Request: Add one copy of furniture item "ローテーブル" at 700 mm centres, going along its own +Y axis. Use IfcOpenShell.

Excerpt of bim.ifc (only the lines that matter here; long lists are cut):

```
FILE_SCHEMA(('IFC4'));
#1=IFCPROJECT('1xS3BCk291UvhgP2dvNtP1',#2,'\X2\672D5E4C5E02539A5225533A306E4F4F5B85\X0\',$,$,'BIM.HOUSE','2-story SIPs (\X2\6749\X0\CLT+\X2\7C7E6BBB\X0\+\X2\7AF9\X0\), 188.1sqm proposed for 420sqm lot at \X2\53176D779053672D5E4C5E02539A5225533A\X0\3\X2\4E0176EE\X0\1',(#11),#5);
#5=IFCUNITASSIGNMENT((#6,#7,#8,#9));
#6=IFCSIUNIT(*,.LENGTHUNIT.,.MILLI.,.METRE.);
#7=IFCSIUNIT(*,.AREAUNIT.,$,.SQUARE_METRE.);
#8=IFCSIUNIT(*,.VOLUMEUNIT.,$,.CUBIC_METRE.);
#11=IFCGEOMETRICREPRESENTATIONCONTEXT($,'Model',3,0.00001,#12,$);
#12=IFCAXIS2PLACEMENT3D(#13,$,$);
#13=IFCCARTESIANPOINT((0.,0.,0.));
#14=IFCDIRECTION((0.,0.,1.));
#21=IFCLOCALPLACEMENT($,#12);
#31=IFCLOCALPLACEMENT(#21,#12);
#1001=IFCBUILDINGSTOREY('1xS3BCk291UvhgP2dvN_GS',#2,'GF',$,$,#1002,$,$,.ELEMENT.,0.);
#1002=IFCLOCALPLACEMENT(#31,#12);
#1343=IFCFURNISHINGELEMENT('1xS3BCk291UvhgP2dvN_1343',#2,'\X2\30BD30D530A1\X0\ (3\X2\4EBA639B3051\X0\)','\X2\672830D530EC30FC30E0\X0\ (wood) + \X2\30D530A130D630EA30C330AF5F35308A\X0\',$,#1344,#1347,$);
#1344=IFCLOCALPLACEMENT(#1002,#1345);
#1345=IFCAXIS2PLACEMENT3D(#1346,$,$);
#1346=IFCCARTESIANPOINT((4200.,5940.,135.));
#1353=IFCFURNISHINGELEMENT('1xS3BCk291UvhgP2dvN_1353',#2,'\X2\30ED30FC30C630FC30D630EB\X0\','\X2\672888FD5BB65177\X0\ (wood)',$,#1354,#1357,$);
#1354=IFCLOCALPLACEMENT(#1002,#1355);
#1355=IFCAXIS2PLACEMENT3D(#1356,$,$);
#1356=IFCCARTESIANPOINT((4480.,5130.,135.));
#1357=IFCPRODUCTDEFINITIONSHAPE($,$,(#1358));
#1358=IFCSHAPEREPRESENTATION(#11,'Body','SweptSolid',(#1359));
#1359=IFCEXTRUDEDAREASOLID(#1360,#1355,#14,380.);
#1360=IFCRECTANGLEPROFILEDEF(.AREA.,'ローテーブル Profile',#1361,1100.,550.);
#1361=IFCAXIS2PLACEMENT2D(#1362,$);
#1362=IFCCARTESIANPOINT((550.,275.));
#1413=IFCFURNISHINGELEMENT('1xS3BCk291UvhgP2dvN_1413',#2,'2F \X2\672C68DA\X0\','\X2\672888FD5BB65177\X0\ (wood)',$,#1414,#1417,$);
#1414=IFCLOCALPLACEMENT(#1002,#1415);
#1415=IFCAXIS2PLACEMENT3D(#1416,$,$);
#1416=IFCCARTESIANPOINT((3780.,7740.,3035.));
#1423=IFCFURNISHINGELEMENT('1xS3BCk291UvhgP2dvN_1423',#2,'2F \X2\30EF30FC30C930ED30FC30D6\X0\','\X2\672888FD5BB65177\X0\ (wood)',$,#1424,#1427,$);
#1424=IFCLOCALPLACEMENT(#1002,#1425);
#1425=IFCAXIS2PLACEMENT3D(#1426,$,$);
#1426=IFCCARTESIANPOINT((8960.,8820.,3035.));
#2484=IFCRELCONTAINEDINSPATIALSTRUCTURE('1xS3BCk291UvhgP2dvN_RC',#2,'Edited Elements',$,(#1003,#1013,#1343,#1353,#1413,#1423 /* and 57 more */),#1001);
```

```python
import ifcopenshell
import ifcopenshell.api.geometry
import ifcopenshell.api.root
import ifcopenshell.util.element
import ifcopenshell.util.placement
import ifcopenshell.util.unit

model = ifcopenshell.open("bim.ifc")
unit_scale = ifcopenshell.util.unit.calculate_unit_scale(model)


def reuse_history(source, copy):
    """copy_class also copies each property set's owner history, people and application; keep the originals."""
    for rel in copy.IsDefinedBy:
        if rel.is_a("IfcRelDefinesByProperties") and (history := rel.RelatingPropertyDefinition.OwnerHistory):
            rel.RelatingPropertyDefinition.OwnerHistory = source.OwnerHistory
            ifcopenshell.util.element.remove_deep2(model, history)


source = model.by_id(1353)
base = ifcopenshell.util.placement.get_local_placement(source.ObjectPlacement)
step = base[:3, 1] * 0.7 / unit_scale

for i in range(1, 2):
    copy = ifcopenshell.api.root.copy_class(model, product=source)
    copy.Representation = ifcopenshell.util.element.copy_deep(
        model, source.Representation, exclude=["IfcGeometricRepresentationContext", "IfcRepresentationMap"]
    )
    reuse_history(source, copy)
    matrix = base.copy()
    matrix[:3, 3] += i * step
    print("added at", matrix[:3, 3].round(3) + 0.0)
    ifcopenshell.api.geometry.edit_object_placement(model, product=copy, matrix=matrix, is_si=False)

model.write("bim-out.ifc")
```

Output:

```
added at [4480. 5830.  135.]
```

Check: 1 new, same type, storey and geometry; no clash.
